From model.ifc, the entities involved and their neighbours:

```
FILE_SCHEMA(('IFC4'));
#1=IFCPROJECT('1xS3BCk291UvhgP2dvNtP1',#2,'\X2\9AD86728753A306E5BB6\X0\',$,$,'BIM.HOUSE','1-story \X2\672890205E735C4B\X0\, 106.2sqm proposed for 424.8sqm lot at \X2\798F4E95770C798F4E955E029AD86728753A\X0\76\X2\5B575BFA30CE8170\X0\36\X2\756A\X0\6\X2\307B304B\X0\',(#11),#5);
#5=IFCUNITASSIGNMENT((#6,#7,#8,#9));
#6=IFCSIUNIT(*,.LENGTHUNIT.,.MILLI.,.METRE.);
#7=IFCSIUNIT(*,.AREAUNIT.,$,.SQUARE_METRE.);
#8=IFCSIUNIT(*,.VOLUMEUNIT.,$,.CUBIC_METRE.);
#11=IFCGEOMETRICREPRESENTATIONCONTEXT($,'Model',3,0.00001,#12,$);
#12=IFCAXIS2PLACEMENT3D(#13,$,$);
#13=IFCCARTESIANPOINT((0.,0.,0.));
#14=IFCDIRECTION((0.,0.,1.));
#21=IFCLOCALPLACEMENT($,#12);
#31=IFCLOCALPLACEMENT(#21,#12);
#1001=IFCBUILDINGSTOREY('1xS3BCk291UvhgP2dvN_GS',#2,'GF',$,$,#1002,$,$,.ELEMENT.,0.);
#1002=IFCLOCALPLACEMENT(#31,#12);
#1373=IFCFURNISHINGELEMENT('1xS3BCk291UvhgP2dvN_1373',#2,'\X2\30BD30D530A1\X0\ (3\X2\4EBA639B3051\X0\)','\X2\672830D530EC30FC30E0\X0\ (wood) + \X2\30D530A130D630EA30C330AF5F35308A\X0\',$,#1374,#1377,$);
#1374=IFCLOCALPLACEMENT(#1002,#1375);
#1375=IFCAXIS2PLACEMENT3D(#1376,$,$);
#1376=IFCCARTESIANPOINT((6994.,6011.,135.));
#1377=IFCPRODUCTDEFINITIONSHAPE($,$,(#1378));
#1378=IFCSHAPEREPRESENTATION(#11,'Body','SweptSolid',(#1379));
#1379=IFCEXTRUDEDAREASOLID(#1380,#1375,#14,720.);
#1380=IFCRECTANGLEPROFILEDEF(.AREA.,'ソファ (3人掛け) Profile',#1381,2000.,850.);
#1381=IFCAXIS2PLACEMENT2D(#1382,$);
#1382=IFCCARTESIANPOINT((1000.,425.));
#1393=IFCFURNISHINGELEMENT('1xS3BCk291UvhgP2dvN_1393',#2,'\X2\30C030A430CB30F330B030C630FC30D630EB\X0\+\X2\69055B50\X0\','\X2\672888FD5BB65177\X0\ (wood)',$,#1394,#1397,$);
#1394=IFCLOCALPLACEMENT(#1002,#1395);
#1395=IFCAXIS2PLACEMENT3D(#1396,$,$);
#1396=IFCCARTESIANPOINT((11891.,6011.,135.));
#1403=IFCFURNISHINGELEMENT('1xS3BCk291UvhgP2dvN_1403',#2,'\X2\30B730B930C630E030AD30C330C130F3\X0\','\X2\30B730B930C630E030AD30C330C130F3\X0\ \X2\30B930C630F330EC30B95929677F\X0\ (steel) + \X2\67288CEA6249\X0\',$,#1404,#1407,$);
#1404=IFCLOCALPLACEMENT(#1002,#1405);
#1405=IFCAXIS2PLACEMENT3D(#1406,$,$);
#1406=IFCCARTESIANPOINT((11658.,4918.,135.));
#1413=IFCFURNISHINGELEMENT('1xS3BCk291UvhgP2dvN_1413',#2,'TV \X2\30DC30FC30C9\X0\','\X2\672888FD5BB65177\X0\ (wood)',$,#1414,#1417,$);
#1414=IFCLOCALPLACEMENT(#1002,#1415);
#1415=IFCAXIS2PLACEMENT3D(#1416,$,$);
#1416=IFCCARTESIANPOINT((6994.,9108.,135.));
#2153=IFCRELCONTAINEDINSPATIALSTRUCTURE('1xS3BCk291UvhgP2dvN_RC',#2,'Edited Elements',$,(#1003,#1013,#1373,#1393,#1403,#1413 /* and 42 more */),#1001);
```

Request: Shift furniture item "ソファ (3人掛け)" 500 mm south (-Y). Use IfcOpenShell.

```python
import ifcopenshell
import ifcopenshell.api.geometry
import ifcopenshell.util.placement

model = ifcopenshell.open("model.ifc")

item = model.by_guid("1xS3BCk291UvhgP2dvN_1373")
matrix = ifcopenshell.util.placement.get_local_placement(item.ObjectPlacement)
matrix[1, 3] -= 500.0
ifcopenshell.api.geometry.edit_object_placement(model, product=item, matrix=matrix, is_si=False)

print(ifcopenshell.util.placement.get_local_placement(item.ObjectPlacement).round(3) + 0.0)

model.write("model_v2.ifc")
```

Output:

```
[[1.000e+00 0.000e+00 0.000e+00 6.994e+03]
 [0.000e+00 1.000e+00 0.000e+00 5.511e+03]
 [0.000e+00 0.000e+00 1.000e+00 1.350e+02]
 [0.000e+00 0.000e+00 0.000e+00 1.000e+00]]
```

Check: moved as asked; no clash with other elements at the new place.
